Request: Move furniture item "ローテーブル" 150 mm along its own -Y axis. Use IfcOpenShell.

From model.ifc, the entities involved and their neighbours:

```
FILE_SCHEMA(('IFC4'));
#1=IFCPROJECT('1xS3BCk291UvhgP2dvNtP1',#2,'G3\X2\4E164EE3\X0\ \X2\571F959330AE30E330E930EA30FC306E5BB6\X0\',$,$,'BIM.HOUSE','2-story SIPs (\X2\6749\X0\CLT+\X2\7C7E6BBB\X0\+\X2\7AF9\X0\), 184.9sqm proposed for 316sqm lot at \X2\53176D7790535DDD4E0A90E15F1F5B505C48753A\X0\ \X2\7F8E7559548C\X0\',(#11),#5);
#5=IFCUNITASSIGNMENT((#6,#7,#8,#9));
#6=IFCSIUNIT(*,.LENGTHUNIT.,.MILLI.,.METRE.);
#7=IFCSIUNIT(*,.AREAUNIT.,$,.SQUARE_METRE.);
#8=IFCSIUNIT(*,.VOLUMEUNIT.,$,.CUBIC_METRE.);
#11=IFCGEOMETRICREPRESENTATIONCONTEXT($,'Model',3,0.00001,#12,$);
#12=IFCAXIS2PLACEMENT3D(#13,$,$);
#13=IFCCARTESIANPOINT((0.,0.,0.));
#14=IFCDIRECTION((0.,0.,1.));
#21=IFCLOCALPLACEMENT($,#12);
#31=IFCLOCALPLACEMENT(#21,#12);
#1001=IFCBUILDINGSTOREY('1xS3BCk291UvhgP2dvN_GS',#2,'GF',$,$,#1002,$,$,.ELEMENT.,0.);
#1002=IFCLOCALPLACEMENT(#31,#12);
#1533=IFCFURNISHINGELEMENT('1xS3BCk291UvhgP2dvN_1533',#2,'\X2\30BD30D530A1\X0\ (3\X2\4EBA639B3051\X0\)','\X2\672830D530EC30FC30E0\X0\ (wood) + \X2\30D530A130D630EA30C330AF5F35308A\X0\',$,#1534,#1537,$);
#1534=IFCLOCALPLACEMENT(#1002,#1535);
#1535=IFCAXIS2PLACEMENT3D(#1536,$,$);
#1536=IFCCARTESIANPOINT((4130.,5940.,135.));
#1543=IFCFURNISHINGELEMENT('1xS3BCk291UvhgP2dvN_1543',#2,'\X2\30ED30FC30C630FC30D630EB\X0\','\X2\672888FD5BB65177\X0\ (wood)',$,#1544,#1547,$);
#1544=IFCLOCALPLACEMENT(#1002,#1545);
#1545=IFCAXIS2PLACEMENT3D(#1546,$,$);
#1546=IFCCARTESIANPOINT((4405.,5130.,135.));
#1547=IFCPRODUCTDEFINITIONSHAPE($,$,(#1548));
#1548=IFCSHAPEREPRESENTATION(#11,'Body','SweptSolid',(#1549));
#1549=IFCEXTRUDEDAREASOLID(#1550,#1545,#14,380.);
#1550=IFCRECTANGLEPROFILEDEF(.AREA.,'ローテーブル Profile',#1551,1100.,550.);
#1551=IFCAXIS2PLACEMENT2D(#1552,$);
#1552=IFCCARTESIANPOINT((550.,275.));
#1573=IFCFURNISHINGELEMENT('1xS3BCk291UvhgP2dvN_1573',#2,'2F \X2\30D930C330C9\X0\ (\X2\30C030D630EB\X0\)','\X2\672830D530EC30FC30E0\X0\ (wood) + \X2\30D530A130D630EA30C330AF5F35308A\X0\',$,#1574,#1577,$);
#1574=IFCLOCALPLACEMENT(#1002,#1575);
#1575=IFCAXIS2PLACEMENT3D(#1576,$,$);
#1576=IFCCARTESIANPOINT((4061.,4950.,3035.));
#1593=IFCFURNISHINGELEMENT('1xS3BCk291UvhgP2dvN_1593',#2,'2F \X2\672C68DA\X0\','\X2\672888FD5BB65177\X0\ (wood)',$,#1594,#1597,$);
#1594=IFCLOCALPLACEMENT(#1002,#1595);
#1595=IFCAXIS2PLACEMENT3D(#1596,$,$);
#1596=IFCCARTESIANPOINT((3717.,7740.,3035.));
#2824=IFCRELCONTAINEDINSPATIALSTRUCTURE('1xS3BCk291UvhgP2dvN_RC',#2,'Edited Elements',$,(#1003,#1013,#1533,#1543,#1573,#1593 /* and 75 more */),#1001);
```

```python
import ifcopenshell
import ifcopenshell.api.geometry
import ifcopenshell.util.placement
import ifcopenshell.util.unit

model = ifcopenshell.open("model.ifc")
unit_scale = ifcopenshell.util.unit.calculate_unit_scale(model)

item = model.by_guid("1xS3BCk291UvhgP2dvN_1543")
matrix = ifcopenshell.util.placement.get_local_placement(item.ObjectPlacement)
matrix[:3, 3] -= matrix[:3, 1] * 0.15 / unit_scale
ifcopenshell.api.geometry.edit_object_placement(model, product=item, matrix=matrix, is_si=False)

print(ifcopenshell.util.placement.get_local_placement(item.ObjectPlacement).round(3) + 0.0)

model.write("model_v2.ifc")
```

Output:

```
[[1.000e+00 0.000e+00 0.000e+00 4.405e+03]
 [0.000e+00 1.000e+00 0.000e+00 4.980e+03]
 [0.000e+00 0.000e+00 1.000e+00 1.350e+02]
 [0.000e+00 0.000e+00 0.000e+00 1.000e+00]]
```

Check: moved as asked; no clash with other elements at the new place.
